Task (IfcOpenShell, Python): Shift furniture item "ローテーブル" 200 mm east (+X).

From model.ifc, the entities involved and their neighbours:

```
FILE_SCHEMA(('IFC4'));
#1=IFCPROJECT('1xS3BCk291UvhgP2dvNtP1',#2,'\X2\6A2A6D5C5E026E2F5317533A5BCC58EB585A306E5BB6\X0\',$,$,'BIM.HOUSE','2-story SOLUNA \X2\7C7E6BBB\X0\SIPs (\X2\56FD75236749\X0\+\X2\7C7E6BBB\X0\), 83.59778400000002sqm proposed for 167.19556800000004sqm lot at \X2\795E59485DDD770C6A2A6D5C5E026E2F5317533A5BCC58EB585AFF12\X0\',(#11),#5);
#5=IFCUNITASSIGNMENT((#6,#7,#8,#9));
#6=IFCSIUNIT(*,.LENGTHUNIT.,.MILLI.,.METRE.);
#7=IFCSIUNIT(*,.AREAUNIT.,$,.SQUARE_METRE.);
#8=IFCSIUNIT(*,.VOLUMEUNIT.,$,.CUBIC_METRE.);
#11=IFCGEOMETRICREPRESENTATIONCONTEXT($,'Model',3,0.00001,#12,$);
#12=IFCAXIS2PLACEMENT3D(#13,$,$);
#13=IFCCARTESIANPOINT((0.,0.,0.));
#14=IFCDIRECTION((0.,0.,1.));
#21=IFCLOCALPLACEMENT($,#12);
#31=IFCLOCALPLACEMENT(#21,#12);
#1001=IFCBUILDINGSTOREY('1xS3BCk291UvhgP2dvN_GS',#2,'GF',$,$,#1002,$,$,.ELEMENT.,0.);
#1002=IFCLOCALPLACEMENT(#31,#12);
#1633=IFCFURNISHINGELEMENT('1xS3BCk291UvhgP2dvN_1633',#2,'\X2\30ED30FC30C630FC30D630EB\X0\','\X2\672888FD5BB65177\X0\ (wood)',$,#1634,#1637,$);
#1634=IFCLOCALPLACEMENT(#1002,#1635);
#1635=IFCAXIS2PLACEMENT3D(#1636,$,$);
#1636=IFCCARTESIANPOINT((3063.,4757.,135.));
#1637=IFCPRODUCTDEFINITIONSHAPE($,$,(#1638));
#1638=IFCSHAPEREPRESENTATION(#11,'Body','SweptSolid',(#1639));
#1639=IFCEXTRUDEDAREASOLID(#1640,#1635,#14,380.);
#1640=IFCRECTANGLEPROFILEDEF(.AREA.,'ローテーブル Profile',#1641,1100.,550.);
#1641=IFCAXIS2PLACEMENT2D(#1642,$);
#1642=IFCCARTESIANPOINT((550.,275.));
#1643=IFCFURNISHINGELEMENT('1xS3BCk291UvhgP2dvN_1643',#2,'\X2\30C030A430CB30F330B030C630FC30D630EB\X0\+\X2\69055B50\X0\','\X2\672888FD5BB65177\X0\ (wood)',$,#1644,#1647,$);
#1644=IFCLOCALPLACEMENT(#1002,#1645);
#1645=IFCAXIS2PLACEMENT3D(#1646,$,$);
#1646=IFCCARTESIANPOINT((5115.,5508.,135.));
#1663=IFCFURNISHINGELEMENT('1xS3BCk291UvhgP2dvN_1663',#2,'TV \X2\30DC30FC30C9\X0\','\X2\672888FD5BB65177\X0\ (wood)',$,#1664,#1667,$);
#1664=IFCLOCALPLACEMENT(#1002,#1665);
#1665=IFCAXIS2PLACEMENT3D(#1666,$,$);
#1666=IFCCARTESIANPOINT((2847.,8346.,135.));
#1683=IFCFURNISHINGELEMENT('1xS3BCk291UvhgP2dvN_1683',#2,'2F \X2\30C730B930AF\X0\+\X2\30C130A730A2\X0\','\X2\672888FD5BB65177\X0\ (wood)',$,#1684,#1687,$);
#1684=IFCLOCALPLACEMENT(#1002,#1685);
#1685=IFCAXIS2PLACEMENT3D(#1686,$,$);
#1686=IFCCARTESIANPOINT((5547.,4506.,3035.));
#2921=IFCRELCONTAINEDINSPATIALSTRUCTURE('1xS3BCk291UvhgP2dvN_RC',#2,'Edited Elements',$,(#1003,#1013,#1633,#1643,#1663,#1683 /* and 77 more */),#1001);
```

```python
import ifcopenshell
import ifcopenshell.api.geometry
import ifcopenshell.util.placement
import ifcopenshell.util.unit

model = ifcopenshell.open("model.ifc")
unit_scale = ifcopenshell.util.unit.calculate_unit_scale(model)

item = model.by_guid("1xS3BCk291UvhgP2dvN_1633")
matrix = ifcopenshell.util.placement.get_local_placement(item.ObjectPlacement)
matrix[0, 3] += 0.2 / unit_scale
ifcopenshell.api.geometry.edit_object_placement(model, product=item, matrix=matrix, is_si=False)

print(ifcopenshell.util.placement.get_local_placement(item.ObjectPlacement).round(3) + 0.0)

model.write("model_updated.ifc")
```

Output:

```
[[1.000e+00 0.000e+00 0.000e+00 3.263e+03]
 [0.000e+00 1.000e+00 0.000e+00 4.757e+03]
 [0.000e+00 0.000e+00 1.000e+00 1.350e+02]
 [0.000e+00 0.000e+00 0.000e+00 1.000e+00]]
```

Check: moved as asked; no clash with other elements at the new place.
